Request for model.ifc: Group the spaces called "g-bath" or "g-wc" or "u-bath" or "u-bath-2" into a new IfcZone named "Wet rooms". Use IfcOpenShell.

First a look at what the model holds.

```python
import ifcopenshell

model = ifcopenshell.open("model.ifc")
print(model.schema)
seen = {}
for space in model.by_type("IfcSpace"):
    seen[space.LongName] = seen.get(space.LongName, 0) + 1
for name, count in sorted(seen.items(), key=str):
    print(count, "x", name)
print("zones:", [z.Name for z in model.by_type("IfcZone")][:20])
```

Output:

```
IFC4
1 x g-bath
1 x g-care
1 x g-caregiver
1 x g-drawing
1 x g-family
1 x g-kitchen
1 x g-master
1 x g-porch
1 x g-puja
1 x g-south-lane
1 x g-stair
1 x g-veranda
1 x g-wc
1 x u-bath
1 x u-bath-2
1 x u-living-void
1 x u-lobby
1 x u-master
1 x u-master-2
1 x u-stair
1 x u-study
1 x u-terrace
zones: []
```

```python
import ifcopenshell
import ifcopenshell.api.group
import ifcopenshell.api.root

model = ifcopenshell.open("model.ifc")

names = {"g-bath", "g-wc", "u-bath", "u-bath-2"}
spaces = [s for s in model.by_type("IfcSpace") if s.LongName in names]

zone = ifcopenshell.api.root.create_entity(model, ifc_class="IfcZone", name="Wet rooms")
ifcopenshell.api.group.assign_group(model, products=spaces, group=zone)
print(len(spaces), "spaces in", zone.Name)

model.write("model_v2.ifc")
```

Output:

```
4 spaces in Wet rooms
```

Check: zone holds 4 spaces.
